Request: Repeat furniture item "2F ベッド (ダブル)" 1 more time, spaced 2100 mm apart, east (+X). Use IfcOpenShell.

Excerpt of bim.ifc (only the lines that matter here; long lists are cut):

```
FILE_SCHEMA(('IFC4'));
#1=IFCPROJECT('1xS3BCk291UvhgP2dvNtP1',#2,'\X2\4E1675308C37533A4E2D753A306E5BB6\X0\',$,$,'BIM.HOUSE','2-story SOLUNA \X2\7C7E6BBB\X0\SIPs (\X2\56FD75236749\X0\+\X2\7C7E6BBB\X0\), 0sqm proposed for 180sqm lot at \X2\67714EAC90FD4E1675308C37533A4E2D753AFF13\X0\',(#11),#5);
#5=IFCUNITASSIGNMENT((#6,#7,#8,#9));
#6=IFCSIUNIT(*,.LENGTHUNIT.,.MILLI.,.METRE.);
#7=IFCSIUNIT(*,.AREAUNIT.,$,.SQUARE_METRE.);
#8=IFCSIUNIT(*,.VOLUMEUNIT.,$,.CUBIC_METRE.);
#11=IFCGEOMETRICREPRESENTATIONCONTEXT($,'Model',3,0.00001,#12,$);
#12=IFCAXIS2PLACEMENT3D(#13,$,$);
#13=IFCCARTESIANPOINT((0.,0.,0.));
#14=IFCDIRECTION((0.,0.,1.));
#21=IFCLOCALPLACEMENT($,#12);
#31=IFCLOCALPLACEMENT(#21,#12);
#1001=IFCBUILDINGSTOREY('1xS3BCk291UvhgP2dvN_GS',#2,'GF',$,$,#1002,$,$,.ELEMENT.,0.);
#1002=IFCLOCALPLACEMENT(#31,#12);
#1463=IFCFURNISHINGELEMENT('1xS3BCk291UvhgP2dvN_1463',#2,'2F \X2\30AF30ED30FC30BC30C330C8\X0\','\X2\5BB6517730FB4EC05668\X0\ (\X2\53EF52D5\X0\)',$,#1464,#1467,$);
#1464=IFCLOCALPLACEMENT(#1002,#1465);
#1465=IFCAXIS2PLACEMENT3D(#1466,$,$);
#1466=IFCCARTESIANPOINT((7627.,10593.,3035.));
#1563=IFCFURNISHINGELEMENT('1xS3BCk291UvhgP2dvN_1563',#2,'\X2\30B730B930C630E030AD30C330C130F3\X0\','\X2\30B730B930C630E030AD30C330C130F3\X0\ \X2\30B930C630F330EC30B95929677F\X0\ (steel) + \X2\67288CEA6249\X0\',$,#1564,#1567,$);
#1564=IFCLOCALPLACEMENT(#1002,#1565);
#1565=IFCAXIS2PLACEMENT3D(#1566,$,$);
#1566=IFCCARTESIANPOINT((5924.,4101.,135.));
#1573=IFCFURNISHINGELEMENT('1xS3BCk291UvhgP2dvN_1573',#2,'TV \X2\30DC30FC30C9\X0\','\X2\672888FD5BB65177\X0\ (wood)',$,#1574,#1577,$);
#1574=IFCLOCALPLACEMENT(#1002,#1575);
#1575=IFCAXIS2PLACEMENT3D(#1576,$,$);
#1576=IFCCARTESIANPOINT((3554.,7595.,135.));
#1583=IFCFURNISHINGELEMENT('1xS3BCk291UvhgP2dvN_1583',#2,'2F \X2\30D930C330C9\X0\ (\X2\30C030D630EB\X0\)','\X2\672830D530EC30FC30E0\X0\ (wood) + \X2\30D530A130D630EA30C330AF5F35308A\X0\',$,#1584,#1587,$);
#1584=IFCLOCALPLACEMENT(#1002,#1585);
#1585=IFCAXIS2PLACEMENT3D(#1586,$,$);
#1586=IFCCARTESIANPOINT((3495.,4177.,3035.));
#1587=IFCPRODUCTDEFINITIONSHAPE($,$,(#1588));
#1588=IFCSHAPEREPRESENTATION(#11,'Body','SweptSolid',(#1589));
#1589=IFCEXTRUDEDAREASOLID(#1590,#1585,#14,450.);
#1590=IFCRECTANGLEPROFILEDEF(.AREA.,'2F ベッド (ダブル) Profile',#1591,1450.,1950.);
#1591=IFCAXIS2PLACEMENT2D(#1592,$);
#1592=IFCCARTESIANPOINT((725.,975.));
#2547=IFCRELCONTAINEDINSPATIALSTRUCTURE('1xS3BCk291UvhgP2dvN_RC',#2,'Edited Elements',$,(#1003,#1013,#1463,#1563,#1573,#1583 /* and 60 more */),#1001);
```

```python
import numpy as np
import ifcopenshell
import ifcopenshell.api.geometry
import ifcopenshell.api.root
import ifcopenshell.util.element
import ifcopenshell.util.placement
import ifcopenshell.util.unit

model = ifcopenshell.open("bim.ifc")
unit_scale = ifcopenshell.util.unit.calculate_unit_scale(model)


def reuse_history(source, copy):
    """copy_class also copies each property set's owner history, people and application; keep the originals."""
    for rel in copy.IsDefinedBy:
        if rel.is_a("IfcRelDefinesByProperties") and (history := rel.RelatingPropertyDefinition.OwnerHistory):
            rel.RelatingPropertyDefinition.OwnerHistory = source.OwnerHistory
            ifcopenshell.util.element.remove_deep2(model, history)


source = model.by_guid("1xS3BCk291UvhgP2dvN_1583")
base = ifcopenshell.util.placement.get_local_placement(source.ObjectPlacement)
step = np.array([1.0, 0.0, 0.0]) * 2.1 / unit_scale

for i in range(1, 2):
    copy = ifcopenshell.api.root.copy_class(model, product=source)
    copy.Representation = ifcopenshell.util.element.copy_deep(
        model, source.Representation, exclude=["IfcGeometricRepresentationContext", "IfcRepresentationMap"]
    )
    reuse_history(source, copy)
    matrix = base.copy()
    matrix[:3, 3] += i * step
    print("added at", matrix[:3, 3].round(3) + 0.0)
    ifcopenshell.api.geometry.edit_object_placement(model, product=copy, matrix=matrix, is_si=False)

model.write("bim_updated.ifc")
```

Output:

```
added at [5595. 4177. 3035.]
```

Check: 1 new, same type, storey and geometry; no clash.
